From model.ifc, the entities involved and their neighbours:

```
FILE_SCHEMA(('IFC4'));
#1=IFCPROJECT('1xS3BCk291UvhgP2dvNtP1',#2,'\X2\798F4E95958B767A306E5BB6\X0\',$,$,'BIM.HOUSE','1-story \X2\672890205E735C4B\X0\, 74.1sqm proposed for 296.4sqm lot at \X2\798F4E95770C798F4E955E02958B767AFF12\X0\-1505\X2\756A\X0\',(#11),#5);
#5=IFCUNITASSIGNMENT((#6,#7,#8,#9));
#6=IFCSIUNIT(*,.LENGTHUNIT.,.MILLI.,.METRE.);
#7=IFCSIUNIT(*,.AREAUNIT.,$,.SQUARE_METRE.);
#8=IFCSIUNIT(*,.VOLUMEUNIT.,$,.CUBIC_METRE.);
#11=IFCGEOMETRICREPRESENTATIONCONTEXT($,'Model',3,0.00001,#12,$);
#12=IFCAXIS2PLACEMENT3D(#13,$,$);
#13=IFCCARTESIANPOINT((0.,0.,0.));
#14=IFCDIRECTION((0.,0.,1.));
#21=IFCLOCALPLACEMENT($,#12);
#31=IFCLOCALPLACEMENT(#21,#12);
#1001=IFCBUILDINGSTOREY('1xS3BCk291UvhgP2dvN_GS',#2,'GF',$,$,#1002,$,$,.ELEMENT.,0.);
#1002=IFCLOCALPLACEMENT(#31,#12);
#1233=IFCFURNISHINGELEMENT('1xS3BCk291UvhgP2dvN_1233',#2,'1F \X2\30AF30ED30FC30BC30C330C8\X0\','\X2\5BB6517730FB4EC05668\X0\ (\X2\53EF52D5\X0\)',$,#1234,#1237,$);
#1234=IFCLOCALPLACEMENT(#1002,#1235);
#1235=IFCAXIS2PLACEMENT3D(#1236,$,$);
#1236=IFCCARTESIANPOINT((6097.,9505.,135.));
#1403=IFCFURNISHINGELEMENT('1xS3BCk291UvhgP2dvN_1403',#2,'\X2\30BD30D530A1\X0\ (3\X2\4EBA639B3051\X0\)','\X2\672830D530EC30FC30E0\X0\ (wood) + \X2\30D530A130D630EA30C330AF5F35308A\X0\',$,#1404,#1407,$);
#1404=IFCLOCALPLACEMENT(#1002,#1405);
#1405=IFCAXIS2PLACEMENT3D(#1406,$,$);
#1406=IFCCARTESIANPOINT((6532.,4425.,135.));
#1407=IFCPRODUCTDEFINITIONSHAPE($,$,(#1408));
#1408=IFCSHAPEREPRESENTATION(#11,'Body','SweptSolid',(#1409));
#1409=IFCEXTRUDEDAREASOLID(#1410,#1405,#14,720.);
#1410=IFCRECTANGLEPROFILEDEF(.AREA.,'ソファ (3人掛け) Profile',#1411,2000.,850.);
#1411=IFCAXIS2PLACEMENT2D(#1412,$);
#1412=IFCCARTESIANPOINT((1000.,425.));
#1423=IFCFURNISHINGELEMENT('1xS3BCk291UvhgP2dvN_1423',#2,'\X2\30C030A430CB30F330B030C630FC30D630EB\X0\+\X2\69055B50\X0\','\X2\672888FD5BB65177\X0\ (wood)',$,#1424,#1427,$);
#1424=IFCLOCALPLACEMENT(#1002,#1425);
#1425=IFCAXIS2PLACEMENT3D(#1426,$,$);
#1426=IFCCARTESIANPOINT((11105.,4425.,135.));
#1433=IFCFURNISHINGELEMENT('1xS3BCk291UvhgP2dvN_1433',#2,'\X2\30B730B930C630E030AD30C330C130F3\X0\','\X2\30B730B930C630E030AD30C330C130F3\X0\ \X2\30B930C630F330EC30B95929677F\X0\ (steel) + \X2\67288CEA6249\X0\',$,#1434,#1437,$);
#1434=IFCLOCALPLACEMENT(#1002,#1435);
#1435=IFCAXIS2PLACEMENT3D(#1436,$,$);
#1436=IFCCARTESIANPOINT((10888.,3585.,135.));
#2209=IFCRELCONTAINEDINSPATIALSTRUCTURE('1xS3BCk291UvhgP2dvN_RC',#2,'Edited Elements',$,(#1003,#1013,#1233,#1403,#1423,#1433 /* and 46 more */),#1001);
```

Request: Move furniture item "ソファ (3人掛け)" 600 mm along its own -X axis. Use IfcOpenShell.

```python
import ifcopenshell
import ifcopenshell.api.geometry
import ifcopenshell.util.placement
import ifcopenshell.util.unit

model = ifcopenshell.open("model.ifc")
unit_scale = ifcopenshell.util.unit.calculate_unit_scale(model)

item = model.by_guid("1xS3BCk291UvhgP2dvN_1403")
matrix = ifcopenshell.util.placement.get_local_placement(item.ObjectPlacement)
matrix[:3, 3] -= matrix[:3, 0] * 0.6 / unit_scale
ifcopenshell.api.geometry.edit_object_placement(model, product=item, matrix=matrix, is_si=False)

print(ifcopenshell.util.placement.get_local_placement(item.ObjectPlacement).round(3) + 0.0)

model.write("model_v2.ifc")
```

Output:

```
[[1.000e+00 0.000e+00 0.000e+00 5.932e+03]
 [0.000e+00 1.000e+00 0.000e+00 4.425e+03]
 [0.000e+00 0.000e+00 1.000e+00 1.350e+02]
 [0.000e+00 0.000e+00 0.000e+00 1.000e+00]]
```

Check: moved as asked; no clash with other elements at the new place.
